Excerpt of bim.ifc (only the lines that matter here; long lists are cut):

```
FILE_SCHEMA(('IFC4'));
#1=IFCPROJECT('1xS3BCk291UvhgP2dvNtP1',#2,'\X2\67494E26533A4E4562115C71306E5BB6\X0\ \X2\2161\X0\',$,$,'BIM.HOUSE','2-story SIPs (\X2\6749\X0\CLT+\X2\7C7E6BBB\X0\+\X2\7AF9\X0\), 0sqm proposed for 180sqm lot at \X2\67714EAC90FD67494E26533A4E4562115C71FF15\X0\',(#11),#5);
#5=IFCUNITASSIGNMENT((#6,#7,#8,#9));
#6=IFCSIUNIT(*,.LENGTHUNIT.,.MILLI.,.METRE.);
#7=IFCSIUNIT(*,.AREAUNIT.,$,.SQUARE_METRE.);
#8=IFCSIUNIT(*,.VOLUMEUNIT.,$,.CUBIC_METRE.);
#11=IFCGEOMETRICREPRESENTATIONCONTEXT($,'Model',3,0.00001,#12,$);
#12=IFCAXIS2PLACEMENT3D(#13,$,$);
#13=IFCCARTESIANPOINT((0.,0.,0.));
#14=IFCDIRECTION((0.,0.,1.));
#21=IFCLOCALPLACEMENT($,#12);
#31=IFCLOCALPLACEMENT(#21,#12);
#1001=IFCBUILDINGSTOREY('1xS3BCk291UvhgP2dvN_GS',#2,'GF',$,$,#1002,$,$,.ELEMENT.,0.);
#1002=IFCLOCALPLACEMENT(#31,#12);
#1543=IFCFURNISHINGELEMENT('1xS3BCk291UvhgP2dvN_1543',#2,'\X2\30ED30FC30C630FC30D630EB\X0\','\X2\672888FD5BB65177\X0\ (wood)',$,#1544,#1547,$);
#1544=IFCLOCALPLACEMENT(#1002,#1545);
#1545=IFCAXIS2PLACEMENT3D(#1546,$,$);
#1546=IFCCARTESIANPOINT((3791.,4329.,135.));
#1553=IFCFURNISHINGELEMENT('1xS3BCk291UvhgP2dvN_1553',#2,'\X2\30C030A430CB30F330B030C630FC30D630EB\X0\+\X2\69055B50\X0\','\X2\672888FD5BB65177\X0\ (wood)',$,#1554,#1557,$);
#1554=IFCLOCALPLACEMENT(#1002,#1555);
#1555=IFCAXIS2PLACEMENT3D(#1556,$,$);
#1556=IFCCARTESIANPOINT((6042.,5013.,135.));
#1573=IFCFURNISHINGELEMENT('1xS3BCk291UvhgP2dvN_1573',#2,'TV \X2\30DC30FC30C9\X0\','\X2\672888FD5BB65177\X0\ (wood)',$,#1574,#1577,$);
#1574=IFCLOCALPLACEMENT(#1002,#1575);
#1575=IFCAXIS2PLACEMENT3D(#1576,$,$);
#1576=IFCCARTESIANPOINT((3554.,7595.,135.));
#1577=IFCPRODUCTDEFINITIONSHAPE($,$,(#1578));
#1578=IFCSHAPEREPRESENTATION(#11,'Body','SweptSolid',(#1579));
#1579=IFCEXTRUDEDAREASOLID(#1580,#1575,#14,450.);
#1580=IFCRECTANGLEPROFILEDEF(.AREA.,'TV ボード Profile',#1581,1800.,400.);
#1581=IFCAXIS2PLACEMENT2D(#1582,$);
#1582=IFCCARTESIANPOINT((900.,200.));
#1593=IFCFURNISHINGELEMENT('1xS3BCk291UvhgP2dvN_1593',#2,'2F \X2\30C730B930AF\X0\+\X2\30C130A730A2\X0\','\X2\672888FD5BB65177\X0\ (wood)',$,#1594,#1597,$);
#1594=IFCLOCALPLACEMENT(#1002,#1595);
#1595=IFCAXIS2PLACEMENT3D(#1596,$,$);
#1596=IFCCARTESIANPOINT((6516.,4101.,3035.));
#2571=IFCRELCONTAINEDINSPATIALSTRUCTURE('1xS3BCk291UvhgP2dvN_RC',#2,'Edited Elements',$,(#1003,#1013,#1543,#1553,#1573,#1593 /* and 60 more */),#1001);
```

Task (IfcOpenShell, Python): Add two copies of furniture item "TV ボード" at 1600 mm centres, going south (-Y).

```python
import numpy as np
import ifcopenshell
import ifcopenshell.api.geometry
import ifcopenshell.api.root
import ifcopenshell.util.element
import ifcopenshell.util.placement

model = ifcopenshell.open("bim.ifc")


def reuse_history(source, copy):
    """copy_class also copies each property set's owner history, people and application; keep the originals."""
    for rel in copy.IsDefinedBy:
        if rel.is_a("IfcRelDefinesByProperties") and (history := rel.RelatingPropertyDefinition.OwnerHistory):
            rel.RelatingPropertyDefinition.OwnerHistory = source.OwnerHistory
            ifcopenshell.util.element.remove_deep2(model, history)


source = model.by_guid("1xS3BCk291UvhgP2dvN_1573")
base = ifcopenshell.util.placement.get_local_placement(source.ObjectPlacement)
step = np.array([0.0, -1.0, 0.0]) * 1600.0

for i in range(1, 3):
    copy = ifcopenshell.api.root.copy_class(model, product=source)
    copy.Representation = ifcopenshell.util.element.copy_deep(
        model, source.Representation, exclude=["IfcGeometricRepresentationContext", "IfcRepresentationMap"]
    )
    reuse_history(source, copy)
    matrix = base.copy()
    matrix[:3, 3] += i * step
    print("added at", matrix[:3, 3].round(3) + 0.0)
    ifcopenshell.api.geometry.edit_object_placement(model, product=copy, matrix=matrix, is_si=False)

model.write("bim_edited.ifc")
```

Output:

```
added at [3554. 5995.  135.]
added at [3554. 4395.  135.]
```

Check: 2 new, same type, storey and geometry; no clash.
